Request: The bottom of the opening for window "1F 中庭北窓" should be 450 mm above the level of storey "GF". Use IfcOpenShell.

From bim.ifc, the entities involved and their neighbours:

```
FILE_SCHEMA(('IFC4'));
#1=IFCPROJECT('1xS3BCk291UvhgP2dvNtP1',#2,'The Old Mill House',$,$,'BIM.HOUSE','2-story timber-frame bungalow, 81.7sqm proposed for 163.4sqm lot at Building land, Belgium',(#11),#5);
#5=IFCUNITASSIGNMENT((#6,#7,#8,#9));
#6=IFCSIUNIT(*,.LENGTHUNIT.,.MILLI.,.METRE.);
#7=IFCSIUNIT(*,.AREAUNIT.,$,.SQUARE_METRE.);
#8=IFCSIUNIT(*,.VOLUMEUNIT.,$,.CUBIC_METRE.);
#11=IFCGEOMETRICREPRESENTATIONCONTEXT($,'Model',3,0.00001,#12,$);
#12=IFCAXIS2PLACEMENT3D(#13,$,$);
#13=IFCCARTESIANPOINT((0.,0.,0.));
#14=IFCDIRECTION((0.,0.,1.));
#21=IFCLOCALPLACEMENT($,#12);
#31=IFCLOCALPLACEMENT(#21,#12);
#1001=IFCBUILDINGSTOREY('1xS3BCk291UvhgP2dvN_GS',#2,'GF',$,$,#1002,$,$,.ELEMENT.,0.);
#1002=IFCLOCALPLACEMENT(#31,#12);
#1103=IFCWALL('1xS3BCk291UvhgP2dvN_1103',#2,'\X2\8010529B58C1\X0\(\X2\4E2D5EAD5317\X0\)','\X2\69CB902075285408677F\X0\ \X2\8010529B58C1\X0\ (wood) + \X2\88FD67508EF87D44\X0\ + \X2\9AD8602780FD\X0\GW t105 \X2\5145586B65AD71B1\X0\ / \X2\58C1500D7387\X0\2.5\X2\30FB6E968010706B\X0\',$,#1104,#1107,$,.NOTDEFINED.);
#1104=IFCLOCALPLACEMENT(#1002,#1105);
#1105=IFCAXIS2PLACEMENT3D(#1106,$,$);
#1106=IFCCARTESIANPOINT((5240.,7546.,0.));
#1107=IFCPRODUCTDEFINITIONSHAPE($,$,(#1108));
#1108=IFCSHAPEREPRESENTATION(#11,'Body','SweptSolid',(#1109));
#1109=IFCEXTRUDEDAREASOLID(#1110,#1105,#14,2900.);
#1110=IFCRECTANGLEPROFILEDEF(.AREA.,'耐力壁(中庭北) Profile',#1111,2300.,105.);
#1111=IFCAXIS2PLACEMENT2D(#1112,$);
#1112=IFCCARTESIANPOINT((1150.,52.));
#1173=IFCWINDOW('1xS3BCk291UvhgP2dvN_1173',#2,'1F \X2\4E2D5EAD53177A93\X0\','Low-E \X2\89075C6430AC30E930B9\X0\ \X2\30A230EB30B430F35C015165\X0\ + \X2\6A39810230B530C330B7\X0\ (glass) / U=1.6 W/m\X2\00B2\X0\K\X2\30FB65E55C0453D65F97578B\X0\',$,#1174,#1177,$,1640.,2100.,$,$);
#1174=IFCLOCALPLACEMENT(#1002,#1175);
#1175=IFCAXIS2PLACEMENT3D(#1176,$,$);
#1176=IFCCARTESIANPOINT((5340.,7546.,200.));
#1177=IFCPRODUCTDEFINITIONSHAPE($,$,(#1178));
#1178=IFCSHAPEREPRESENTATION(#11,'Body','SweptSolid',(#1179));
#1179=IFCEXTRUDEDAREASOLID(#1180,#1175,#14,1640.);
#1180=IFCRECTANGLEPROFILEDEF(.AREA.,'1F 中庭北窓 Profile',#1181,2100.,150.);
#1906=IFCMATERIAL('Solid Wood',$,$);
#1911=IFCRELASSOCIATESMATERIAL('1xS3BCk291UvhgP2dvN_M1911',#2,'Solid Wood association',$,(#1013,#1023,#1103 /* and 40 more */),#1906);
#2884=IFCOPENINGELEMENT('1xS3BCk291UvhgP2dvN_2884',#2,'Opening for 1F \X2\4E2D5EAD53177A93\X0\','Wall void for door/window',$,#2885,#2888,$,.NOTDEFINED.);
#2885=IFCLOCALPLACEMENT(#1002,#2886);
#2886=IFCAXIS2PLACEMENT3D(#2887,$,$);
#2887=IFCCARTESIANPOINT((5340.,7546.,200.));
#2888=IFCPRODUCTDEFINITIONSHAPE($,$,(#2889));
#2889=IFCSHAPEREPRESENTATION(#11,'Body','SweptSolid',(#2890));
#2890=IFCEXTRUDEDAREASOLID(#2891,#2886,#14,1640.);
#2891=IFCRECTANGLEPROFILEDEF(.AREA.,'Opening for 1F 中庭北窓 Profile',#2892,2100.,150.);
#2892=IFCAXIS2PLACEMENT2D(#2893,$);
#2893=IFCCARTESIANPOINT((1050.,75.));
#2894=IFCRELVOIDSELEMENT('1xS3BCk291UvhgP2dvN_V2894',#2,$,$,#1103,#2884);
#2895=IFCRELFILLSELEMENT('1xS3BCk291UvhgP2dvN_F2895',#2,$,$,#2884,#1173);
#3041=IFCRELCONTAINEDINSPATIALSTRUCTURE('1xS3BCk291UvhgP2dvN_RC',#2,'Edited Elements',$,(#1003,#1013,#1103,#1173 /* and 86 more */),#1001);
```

```python
import numpy as np
import ifcopenshell
import ifcopenshell.api.geometry
import ifcopenshell.geom
import ifcopenshell.util.element
import ifcopenshell.util.placement
import ifcopenshell.util.shape
import ifcopenshell.util.unit

model = ifcopenshell.open("bim.ifc")
unit_scale = ifcopenshell.util.unit.calculate_unit_scale(model)

window = model.by_guid("1xS3BCk291UvhgP2dvN_1173")
opening = window.FillsVoids[0].RelatingOpeningElement
storey = ifcopenshell.util.element.get_container(window, ifc_class="IfcBuildingStorey")
level = ifcopenshell.util.placement.get_local_placement(storey.ObjectPlacement)[2, 3]

# The opening's origin need not be at the sill, so measure its lowest point.
shape = ifcopenshell.geom.create_shape(ifcopenshell.geom.settings(), opening)
bottom = ifcopenshell.util.shape.get_shape_bottom_elevation(shape, shape.geometry) / unit_scale
dz = level + 0.45 / unit_scale - bottom

shift = np.array([0.0, 0.0, dz])
# The window is not placed relative to its opening, so move both.
for product in (opening, window):
    matrix = ifcopenshell.util.placement.get_local_placement(product.ObjectPlacement)
    matrix[:3, 3] += shift
    ifcopenshell.api.geometry.edit_object_placement(model, product=product, matrix=matrix, is_si=False)

print(f"moved by {dz * unit_scale:+.3f} m")

model.write("bim_updated.ifc")
```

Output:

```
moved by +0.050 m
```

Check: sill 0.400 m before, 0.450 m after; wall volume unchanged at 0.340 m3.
